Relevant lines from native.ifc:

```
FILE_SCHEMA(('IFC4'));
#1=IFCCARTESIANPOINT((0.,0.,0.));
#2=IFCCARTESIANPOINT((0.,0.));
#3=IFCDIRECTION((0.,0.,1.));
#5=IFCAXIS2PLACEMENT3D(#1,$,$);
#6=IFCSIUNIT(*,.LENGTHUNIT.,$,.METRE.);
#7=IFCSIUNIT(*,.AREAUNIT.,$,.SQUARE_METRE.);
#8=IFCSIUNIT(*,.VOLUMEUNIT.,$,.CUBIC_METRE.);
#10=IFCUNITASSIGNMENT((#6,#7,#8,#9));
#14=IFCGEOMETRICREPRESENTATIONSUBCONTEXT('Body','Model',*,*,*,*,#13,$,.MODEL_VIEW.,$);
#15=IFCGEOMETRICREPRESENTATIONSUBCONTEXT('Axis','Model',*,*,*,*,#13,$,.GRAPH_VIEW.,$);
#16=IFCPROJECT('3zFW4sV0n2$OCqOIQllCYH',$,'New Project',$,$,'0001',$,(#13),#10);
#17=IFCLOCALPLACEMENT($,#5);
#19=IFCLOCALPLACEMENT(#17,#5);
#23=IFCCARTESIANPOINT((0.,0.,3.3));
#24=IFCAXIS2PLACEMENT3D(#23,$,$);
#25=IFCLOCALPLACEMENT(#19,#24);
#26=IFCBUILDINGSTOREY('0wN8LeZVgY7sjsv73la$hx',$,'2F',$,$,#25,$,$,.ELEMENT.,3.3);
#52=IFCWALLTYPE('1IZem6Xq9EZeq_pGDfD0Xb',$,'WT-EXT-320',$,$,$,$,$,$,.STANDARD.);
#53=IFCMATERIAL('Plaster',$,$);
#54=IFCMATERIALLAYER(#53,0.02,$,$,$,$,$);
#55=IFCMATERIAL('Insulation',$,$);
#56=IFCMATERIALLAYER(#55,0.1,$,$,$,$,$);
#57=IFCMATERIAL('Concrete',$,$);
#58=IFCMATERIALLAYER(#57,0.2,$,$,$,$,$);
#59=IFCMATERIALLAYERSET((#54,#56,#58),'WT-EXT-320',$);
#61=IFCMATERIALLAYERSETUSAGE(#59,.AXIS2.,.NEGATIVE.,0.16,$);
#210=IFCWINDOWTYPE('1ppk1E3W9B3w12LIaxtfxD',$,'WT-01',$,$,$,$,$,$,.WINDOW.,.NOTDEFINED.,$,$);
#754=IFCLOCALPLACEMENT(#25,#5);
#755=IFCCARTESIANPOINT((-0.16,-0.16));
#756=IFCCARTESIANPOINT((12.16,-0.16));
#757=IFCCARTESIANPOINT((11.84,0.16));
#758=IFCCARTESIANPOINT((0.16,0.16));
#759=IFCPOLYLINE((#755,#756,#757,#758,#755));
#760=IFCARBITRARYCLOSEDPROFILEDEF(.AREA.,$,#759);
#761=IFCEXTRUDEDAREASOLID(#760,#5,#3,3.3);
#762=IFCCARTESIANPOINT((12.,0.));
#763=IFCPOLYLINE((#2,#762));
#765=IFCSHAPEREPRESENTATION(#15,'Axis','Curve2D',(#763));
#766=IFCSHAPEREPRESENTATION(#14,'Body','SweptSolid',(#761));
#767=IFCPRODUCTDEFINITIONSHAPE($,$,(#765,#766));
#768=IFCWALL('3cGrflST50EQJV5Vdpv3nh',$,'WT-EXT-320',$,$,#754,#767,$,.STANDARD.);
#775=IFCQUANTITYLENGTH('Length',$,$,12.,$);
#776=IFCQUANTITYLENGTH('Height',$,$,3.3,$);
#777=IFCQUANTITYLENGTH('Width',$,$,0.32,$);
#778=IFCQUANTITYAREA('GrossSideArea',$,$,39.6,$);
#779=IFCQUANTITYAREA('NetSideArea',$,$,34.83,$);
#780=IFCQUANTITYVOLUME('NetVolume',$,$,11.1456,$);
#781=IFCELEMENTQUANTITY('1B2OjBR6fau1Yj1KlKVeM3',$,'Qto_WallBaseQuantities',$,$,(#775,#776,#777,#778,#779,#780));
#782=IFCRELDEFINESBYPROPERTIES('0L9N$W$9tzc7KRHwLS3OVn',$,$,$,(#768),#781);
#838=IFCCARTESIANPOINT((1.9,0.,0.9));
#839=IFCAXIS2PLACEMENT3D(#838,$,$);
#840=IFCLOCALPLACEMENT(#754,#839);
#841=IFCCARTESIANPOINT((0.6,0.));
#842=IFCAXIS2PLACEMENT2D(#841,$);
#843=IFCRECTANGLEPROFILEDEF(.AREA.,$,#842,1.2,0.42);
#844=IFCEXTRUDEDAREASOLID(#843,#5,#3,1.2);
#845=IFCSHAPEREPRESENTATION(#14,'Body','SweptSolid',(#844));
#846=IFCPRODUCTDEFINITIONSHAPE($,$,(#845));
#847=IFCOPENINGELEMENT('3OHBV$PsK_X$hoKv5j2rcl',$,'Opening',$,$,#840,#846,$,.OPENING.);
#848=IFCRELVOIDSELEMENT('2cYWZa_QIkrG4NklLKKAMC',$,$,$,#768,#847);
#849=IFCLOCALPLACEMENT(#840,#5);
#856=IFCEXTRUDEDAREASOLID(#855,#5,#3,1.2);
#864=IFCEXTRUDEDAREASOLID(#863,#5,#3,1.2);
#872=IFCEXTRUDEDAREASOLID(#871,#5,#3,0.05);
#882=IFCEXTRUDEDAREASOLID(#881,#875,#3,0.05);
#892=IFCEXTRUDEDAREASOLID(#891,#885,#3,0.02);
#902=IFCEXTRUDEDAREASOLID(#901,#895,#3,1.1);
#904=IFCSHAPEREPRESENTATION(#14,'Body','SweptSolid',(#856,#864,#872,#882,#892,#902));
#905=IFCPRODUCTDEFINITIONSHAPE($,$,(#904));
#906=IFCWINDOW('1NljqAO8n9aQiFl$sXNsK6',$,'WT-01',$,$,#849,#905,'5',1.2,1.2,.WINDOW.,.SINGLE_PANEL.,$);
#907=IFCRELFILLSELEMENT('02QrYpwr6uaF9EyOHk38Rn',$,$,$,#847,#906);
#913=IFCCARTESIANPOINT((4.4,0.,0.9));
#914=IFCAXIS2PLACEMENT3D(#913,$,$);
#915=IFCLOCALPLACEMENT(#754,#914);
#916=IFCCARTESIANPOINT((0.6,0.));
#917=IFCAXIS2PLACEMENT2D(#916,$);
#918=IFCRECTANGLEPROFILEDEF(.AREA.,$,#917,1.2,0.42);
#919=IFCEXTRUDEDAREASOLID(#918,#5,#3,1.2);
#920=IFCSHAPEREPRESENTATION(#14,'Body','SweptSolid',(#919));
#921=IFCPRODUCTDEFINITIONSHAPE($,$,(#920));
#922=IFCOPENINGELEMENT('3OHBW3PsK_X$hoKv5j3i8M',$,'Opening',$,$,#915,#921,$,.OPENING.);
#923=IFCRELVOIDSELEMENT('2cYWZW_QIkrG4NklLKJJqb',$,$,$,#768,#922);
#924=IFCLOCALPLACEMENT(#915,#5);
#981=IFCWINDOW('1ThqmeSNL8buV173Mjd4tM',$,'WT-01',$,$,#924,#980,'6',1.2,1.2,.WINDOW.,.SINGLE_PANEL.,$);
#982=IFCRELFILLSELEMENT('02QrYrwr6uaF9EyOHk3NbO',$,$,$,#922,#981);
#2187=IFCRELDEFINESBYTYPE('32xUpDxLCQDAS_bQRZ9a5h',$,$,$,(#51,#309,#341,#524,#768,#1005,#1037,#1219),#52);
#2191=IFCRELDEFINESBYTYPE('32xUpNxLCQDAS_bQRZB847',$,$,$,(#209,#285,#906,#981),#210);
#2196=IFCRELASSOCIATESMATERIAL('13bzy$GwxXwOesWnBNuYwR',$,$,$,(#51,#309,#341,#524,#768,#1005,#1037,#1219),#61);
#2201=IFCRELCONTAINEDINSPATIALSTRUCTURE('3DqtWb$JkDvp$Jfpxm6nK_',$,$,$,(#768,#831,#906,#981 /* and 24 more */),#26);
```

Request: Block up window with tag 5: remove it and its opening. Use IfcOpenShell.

```python
import ifcopenshell
import ifcopenshell.api.feature
import ifcopenshell.api.pset
import ifcopenshell.api.root
import ifcopenshell.geom
import ifcopenshell.util.element
import ifcopenshell.util.shape
import ifcopenshell.util.unit

model = ifcopenshell.open("native.ifc")
area_scale = ifcopenshell.util.unit.calculate_unit_scale(model, "AREAUNIT")
volume_scale = ifcopenshell.util.unit.calculate_unit_scale(model, "VOLUMEUNIT")
settings = ifcopenshell.geom.settings()


def volume(element):
    """Net volume in cubic metres, openings subtracted."""
    shape = ifcopenshell.geom.create_shape(settings, element)
    return ifcopenshell.util.shape.get_volume(shape.geometry)


window = model.by_guid("1NljqAO8n9aQiFl$sXNsK6")
opening = window.FillsVoids[0].RelatingOpeningElement
wall = opening.VoidsElements[0].RelatingBuildingElement
before = volume(wall)

ifcopenshell.api.root.remove_product(model, product=window)
ifcopenshell.api.feature.remove_feature(model, feature=opening)

after = volume(wall)
thickness = 0.32  # wall thickness in metres

# Update the wall's stored quantities.
qto = model.by_id(ifcopenshell.util.element.get_pset(wall, "Qto_WallBaseQuantities", should_inherit=False)["id"])
ifcopenshell.api.pset.edit_qto(model, qto=qto, properties={
    "NetSideArea": after / thickness / area_scale,
    "NetVolume": after / volume_scale,
})

print(f"wall volume {before:.3f} -> {after:.3f} m3")

model.write("native_edited.ifc")
```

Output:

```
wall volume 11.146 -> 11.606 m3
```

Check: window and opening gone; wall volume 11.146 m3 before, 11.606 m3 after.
